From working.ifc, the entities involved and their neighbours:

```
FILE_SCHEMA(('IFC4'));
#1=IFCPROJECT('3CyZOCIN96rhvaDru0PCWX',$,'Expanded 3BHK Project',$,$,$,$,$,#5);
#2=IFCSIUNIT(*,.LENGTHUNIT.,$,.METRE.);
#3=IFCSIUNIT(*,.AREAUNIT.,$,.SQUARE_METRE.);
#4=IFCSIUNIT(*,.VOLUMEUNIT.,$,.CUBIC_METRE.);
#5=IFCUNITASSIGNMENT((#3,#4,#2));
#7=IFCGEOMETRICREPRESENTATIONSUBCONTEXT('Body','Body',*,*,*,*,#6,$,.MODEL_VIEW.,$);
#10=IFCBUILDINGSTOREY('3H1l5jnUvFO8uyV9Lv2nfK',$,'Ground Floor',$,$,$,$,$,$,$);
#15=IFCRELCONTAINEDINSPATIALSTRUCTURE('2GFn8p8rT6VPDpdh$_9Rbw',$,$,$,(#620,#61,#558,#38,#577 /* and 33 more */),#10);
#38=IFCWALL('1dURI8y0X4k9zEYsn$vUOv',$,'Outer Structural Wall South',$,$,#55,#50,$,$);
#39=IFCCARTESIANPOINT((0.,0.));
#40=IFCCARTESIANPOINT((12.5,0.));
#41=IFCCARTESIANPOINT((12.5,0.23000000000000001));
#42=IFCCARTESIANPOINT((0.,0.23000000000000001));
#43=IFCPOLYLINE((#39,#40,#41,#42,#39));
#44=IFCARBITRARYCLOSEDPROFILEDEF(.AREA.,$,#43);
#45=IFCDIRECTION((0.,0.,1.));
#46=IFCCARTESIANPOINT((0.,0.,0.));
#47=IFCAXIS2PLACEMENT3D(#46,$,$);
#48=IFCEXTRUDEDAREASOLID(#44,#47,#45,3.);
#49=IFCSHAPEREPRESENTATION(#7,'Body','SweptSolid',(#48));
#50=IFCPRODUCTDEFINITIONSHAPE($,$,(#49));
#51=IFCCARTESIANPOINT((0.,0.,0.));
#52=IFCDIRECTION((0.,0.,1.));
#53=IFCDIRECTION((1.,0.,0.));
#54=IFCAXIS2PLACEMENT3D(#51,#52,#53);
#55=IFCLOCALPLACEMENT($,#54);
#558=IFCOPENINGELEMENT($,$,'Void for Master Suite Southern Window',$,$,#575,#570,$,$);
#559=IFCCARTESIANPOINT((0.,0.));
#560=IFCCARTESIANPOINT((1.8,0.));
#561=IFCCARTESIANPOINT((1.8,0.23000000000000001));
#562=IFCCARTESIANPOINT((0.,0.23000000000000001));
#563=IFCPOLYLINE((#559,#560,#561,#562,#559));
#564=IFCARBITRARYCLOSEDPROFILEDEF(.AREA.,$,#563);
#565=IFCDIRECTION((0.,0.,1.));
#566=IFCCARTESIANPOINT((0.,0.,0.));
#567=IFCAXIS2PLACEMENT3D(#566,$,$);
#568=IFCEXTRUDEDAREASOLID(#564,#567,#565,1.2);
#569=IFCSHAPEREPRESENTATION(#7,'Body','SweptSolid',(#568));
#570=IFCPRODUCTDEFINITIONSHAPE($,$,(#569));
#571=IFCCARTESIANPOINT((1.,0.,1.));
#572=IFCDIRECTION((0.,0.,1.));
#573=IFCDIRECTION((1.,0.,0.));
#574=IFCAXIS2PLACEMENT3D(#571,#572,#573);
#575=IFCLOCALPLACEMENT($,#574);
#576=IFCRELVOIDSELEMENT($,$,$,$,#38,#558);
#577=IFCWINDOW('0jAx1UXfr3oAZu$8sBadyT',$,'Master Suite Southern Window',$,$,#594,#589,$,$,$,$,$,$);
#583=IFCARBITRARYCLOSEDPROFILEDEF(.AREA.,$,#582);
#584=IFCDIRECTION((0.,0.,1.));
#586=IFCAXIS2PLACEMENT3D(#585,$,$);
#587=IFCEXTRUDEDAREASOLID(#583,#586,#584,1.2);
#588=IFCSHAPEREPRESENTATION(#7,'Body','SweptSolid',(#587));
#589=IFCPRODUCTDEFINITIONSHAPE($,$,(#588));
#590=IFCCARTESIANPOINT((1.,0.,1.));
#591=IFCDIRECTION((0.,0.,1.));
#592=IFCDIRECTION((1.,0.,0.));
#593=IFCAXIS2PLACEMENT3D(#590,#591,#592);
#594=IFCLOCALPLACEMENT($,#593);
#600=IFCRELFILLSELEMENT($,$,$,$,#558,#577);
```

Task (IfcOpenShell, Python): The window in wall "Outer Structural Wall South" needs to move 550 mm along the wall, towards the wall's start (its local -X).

```python
import ifcopenshell
import ifcopenshell.api.geometry
import ifcopenshell.util.placement

model = ifcopenshell.open("working.ifc")

window = model.by_guid("0jAx1UXfr3oAZu$8sBadyT")
opening = window.FillsVoids[0].RelatingOpeningElement
wall = opening.VoidsElements[0].RelatingBuildingElement

wall_matrix = ifcopenshell.util.placement.get_local_placement(wall.ObjectPlacement)
shift = wall_matrix[:3, 0] * -0.55
before = ifcopenshell.util.placement.get_local_placement(window.ObjectPlacement)[:3, 3].copy()

# The window is not placed relative to its opening, so move both.
for product in (opening, window):
    matrix = ifcopenshell.util.placement.get_local_placement(product.ObjectPlacement)
    matrix[:3, 3] += shift
    ifcopenshell.api.geometry.edit_object_placement(model, product=product, matrix=matrix, is_si=False)

after = ifcopenshell.util.placement.get_local_placement(window.ObjectPlacement)[:3, 3]
print("window moved by", (after - before).round(3) + 0.0)

model.write("working-out.ifc")
```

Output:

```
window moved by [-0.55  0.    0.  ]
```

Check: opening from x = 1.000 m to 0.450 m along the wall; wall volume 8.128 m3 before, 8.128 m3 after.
